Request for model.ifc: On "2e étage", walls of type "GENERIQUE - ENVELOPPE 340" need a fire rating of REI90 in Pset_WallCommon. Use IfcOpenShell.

First a look at what the model holds.

```python
import ifcopenshell
import ifcopenshell.util.element

model = ifcopenshell.open("model.ifc")
print(model.schema)
storey = next(s for s in model.by_type("IfcBuildingStorey") if s.Name == "2e étage")
walls = [e for e in ifcopenshell.util.element.get_decomposition(storey) if e.is_a("IfcWall")]
seen = {}
for e in walls:
    element_type = ifcopenshell.util.element.get_type(e)
    key = (element_type.Name if element_type != e and element_type else None, ifcopenshell.util.element.get_pset(e, "Pset_WallCommon", "FireRating"))
    seen[key] = seen.get(key, 0) + 1
for (name, value), count in sorted(seen.items(), key=str):
    print(count, "x", name, "|", value)
```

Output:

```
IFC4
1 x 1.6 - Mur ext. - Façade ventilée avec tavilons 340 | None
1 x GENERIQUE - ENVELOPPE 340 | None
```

```python
import ifcopenshell
import ifcopenshell.api.pset
import ifcopenshell.util.element

model = ifcopenshell.open("model.ifc")

storey = next(s for s in model.by_type("IfcBuildingStorey") if s.Name == "2e étage")
walls = [e for e in ifcopenshell.util.element.get_decomposition(storey) if e.is_a("IfcWall")]

count = 0
for e in walls:
    element_type = ifcopenshell.util.element.get_type(e)
    if element_type in (None, e) or element_type.Name != "GENERIQUE - ENVELOPPE 340":
        continue
    # add_pset returns the element's existing set when there is one.
    pset = ifcopenshell.api.pset.add_pset(model, product=e, name="Pset_WallCommon")
    ifcopenshell.api.pset.edit_pset(model, pset=pset, properties={"FireRating": "REI90"})
    count += 1

print(count, "walls updated")

model.write("model_rev.ifc")
```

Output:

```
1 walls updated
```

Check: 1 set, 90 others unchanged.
